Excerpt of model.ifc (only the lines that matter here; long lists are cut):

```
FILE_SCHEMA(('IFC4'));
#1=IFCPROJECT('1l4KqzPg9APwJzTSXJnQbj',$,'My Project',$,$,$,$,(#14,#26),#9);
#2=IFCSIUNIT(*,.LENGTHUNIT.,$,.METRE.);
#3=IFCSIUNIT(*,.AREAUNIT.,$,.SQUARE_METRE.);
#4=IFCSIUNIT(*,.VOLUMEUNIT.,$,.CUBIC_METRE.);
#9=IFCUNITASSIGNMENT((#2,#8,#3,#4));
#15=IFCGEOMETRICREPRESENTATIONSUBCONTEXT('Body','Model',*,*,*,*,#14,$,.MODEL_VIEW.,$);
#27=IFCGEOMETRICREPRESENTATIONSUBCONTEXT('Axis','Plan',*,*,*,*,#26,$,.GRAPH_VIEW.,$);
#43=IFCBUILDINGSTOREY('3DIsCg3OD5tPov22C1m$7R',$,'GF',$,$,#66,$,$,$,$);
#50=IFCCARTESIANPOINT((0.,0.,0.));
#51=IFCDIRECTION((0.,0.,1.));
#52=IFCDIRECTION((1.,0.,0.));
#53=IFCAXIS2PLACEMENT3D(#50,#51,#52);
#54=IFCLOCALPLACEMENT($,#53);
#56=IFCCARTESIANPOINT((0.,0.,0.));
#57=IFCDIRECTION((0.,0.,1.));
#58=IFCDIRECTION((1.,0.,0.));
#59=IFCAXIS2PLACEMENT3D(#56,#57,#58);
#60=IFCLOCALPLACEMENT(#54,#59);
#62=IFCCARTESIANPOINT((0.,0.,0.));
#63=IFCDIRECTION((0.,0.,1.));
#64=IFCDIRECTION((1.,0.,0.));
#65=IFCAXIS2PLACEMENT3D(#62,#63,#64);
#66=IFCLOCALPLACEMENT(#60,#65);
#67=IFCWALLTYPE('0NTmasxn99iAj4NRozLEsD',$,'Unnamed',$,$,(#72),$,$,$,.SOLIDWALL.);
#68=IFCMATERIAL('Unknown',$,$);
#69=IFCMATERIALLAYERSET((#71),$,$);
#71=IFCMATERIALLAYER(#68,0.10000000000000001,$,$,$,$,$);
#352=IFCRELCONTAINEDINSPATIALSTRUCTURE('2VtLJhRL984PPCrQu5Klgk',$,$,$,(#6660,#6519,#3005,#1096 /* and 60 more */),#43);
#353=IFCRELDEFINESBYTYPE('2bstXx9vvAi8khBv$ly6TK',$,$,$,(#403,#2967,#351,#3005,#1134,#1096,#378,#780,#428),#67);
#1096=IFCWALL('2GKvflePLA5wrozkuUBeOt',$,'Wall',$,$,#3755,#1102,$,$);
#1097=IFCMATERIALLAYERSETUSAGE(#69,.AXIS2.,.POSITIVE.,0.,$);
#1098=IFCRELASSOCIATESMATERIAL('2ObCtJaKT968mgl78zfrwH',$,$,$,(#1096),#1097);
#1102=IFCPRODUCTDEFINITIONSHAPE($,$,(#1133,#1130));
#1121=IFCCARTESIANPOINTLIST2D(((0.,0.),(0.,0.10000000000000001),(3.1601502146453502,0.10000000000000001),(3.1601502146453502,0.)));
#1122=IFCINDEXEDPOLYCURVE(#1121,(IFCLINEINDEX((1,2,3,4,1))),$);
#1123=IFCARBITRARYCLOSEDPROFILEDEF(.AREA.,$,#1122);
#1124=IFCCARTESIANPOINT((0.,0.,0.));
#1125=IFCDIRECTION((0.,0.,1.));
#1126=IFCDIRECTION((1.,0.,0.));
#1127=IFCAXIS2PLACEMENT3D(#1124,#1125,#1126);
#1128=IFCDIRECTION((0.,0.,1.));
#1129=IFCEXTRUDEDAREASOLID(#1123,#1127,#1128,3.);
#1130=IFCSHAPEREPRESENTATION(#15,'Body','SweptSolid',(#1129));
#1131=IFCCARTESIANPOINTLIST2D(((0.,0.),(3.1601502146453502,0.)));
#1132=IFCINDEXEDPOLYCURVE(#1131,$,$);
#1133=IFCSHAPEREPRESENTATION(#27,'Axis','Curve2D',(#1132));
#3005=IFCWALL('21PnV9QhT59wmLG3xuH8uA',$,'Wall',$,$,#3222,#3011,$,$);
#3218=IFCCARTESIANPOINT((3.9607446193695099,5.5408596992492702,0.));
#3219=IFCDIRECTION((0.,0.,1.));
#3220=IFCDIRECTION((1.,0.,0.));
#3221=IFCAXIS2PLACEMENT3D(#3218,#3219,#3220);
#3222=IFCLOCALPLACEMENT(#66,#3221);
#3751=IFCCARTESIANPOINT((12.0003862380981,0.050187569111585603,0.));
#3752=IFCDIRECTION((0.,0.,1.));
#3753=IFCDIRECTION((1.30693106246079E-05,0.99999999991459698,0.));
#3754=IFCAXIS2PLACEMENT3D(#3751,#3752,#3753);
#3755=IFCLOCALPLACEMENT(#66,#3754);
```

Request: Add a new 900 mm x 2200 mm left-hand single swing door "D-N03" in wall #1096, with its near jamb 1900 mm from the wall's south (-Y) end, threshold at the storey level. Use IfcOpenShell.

```python
import numpy as np
import ifcopenshell
import ifcopenshell.api.feature
import ifcopenshell.api.geometry
import ifcopenshell.api.root
import ifcopenshell.api.spatial
import ifcopenshell.geom
import ifcopenshell.util.element
import ifcopenshell.util.placement
import ifcopenshell.util.representation
import ifcopenshell.util.shape
import ifcopenshell.util.unit

model = ifcopenshell.open("model.ifc")
unit_scale = ifcopenshell.util.unit.calculate_unit_scale(model)
settings = ifcopenshell.geom.settings()


def volume(element):
    """Net volume in cubic metres, openings subtracted."""
    shape = ifcopenshell.geom.create_shape(settings, element)
    return ifcopenshell.util.shape.get_volume(shape.geometry)


wall = model.by_guid("2GKvflePLA5wrozkuUBeOt")
storey = ifcopenshell.util.element.get_container(wall, ifc_class="IfcBuildingStorey")
context = ifcopenshell.util.representation.get_context(model, "Model", "Body", "MODEL_VIEW")
before = volume(wall)

width, height, from_end, sill = 0.9, 2.2, 1.9, 0.0  # metres

# The wall runs along its own X axis, and the end named is its -X end.
wall_shape = ifcopenshell.geom.create_shape(settings, wall)
x, y, z = ifcopenshell.util.shape.get_vertices(wall_shape.geometry).T
start = x.min() + from_end
face, thickness = float(y.min()), float(y.max() - y.min())
wall_matrix = ifcopenshell.util.placement.get_local_placement(wall.ObjectPlacement)
level = ifcopenshell.util.placement.get_local_placement(storey.ObjectPlacement)[2, 3]


def in_wall(x, y):
    """Placement at x, y metres in the wall's axes, at sill height."""
    matrix = wall_matrix.copy()
    matrix[:, 3] = wall_matrix @ np.array([x / unit_scale, y / unit_scale, 0.0, 1.0])
    matrix[2, 3] = level + sill / unit_scale
    return matrix


# Opening: a box that overshoots both wall faces by 50 mm.
opening = ifcopenshell.api.root.create_entity(model, ifc_class="IfcOpeningElement", predefined_type="OPENING")
box = ifcopenshell.api.geometry.add_wall_representation(
    model, context=context, length=width, height=height, thickness=thickness + 0.1
)
ifcopenshell.api.geometry.assign_representation(model, product=opening, representation=box)
ifcopenshell.api.geometry.edit_object_placement(model, product=opening, matrix=in_wall(start, face - 0.05), is_si=False)
ifcopenshell.api.feature.add_feature(model, feature=opening, element=wall)

door = ifcopenshell.api.root.create_entity(model, ifc_class="IfcDoor", name="D-N03", predefined_type="DOOR")
door.OverallWidth, door.OverallHeight = width / unit_scale, height / unit_scale
door.OperationType = "SINGLE_SWING_LEFT"
body = ifcopenshell.api.geometry.add_door_representation(
    model,
    context=context,
    overall_width=door.OverallWidth,
    overall_height=door.OverallHeight,
    operation_type="SINGLE_SWING_LEFT",
    lining_properties={"LiningDepth": thickness / unit_scale, "ThresholdDepth": thickness / unit_scale},
)
ifcopenshell.api.geometry.assign_representation(model, product=door, representation=body)
ifcopenshell.api.spatial.assign_container(model, products=[door], relating_structure=storey)
ifcopenshell.api.feature.add_filling(model, opening=opening, element=door)

# The lining spans the wall, so the door starts at the wall face.
ifcopenshell.api.geometry.edit_object_placement(model, product=door, matrix=in_wall(start, face), is_si=False)

after = volume(wall)

print(f"wall volume {before:.3f} -> {after:.3f} m3")

model.write("model_updated.ifc")
```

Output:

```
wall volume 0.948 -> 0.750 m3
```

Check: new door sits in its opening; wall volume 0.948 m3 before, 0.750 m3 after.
